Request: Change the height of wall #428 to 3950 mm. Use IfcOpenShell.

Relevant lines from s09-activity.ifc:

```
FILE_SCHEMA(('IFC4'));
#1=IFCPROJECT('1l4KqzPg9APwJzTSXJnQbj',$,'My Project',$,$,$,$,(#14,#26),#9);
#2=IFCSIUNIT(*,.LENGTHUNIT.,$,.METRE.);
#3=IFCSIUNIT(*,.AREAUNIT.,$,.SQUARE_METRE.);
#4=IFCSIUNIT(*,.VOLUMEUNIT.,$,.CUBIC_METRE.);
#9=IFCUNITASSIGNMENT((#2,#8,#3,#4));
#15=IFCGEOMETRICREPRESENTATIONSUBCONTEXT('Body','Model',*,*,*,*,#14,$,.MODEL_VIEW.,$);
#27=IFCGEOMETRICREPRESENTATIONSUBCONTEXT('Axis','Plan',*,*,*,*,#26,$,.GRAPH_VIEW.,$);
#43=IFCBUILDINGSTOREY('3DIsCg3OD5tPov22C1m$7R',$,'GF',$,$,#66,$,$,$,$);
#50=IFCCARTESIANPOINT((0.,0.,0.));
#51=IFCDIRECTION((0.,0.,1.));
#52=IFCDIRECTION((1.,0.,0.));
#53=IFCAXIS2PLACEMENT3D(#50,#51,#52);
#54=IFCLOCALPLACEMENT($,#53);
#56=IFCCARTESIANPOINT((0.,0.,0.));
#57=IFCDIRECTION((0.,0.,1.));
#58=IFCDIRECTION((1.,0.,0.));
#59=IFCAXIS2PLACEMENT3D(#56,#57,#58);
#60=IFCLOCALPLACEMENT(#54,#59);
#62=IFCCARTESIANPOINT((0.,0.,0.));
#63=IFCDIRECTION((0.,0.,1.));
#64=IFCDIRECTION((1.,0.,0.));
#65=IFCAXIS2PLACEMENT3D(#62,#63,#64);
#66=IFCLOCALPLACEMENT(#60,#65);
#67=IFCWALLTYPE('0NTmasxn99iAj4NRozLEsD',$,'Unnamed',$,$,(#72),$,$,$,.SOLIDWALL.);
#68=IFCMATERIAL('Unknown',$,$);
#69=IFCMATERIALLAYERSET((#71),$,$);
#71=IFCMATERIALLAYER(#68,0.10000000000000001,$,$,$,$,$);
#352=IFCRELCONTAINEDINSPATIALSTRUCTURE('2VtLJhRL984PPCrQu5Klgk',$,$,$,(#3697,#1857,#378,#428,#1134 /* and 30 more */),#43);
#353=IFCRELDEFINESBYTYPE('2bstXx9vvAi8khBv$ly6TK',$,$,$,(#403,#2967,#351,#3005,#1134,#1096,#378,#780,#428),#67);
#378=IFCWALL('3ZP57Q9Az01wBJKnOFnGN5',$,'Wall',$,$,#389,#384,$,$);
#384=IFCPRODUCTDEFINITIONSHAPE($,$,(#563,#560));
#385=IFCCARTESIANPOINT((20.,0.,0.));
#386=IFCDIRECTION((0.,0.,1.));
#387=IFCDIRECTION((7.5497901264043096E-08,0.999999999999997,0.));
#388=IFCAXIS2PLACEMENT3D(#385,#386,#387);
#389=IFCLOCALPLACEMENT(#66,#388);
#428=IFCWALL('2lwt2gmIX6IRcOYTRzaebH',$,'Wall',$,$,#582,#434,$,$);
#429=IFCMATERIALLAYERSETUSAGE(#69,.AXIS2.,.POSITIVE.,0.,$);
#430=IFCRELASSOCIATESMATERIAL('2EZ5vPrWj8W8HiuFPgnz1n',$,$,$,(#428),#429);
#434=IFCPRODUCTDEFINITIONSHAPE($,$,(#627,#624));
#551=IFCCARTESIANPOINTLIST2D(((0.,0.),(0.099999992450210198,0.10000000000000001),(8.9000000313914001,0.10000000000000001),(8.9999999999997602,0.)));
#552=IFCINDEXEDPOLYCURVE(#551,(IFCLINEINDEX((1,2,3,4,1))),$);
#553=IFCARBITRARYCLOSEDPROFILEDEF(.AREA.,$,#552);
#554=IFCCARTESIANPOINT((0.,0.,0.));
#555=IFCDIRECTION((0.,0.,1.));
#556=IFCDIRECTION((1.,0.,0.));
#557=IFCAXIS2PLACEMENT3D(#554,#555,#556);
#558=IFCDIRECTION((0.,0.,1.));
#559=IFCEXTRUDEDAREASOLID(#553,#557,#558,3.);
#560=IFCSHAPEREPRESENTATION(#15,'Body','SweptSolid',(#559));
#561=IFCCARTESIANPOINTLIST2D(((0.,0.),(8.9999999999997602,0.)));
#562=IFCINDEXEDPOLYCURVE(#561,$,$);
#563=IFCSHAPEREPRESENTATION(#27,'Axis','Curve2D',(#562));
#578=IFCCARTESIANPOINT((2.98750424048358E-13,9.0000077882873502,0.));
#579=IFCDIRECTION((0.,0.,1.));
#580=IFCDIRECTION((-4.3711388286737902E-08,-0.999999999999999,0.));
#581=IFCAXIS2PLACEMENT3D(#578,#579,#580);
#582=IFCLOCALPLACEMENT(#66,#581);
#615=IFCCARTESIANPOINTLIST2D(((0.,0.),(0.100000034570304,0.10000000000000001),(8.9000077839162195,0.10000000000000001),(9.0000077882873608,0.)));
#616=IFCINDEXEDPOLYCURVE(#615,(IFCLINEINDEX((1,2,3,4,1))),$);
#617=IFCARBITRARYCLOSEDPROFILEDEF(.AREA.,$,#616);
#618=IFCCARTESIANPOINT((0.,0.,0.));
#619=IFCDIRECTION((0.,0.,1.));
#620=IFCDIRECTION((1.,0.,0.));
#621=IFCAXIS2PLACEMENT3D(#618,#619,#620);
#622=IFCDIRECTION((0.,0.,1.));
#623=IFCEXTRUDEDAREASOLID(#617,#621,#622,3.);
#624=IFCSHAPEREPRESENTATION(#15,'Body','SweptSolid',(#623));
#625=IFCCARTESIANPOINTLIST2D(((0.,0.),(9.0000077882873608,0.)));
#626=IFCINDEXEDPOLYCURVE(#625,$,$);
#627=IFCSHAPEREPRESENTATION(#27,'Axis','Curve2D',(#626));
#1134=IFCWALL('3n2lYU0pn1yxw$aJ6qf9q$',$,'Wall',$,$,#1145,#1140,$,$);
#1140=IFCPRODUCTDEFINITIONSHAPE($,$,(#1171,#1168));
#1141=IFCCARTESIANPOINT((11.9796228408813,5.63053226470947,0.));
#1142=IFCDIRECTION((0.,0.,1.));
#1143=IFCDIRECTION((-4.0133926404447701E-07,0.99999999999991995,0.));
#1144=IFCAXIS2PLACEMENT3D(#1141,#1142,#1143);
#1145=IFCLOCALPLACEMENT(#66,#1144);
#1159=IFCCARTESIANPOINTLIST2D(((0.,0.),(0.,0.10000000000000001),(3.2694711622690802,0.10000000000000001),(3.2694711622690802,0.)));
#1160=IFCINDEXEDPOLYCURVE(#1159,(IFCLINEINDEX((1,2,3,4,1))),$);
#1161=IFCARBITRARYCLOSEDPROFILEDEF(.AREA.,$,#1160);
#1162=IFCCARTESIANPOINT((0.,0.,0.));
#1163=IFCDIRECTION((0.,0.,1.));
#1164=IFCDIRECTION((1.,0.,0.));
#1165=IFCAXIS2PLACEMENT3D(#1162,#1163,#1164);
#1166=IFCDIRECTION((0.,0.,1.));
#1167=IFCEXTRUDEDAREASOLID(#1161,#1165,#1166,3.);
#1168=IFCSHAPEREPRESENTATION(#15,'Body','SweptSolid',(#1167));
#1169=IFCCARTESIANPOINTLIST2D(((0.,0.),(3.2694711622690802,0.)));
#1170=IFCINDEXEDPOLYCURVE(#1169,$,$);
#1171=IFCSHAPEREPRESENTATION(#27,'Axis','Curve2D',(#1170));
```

```python
import ifcopenshell
import ifcopenshell.geom
import ifcopenshell.util.representation
import ifcopenshell.util.shape
import ifcopenshell.util.unit

model = ifcopenshell.open("s09-activity.ifc")
unit_scale = ifcopenshell.util.unit.calculate_unit_scale(model)
settings = ifcopenshell.geom.settings()


def volume(element):
    """Net volume in cubic metres, openings subtracted."""
    shape = ifcopenshell.geom.create_shape(settings, element)
    return ifcopenshell.util.shape.get_volume(shape.geometry)


wall = model.by_guid("2lwt2gmIX6IRcOYTRzaebH")
before = volume(wall)

body = ifcopenshell.util.representation.get_representation(wall, "Model", "Body")
solid = body.Items[0]
old_height = solid.Depth
solid.Depth = 3.95 / unit_scale
after = volume(wall)

print(f"height {old_height:g} -> {solid.Depth:g}, volume {before:.3f} -> {after:.3f} m3")

model.write("s09-activity-out.ifc")
```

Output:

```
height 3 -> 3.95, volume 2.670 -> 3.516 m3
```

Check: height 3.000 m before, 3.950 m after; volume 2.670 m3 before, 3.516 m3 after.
